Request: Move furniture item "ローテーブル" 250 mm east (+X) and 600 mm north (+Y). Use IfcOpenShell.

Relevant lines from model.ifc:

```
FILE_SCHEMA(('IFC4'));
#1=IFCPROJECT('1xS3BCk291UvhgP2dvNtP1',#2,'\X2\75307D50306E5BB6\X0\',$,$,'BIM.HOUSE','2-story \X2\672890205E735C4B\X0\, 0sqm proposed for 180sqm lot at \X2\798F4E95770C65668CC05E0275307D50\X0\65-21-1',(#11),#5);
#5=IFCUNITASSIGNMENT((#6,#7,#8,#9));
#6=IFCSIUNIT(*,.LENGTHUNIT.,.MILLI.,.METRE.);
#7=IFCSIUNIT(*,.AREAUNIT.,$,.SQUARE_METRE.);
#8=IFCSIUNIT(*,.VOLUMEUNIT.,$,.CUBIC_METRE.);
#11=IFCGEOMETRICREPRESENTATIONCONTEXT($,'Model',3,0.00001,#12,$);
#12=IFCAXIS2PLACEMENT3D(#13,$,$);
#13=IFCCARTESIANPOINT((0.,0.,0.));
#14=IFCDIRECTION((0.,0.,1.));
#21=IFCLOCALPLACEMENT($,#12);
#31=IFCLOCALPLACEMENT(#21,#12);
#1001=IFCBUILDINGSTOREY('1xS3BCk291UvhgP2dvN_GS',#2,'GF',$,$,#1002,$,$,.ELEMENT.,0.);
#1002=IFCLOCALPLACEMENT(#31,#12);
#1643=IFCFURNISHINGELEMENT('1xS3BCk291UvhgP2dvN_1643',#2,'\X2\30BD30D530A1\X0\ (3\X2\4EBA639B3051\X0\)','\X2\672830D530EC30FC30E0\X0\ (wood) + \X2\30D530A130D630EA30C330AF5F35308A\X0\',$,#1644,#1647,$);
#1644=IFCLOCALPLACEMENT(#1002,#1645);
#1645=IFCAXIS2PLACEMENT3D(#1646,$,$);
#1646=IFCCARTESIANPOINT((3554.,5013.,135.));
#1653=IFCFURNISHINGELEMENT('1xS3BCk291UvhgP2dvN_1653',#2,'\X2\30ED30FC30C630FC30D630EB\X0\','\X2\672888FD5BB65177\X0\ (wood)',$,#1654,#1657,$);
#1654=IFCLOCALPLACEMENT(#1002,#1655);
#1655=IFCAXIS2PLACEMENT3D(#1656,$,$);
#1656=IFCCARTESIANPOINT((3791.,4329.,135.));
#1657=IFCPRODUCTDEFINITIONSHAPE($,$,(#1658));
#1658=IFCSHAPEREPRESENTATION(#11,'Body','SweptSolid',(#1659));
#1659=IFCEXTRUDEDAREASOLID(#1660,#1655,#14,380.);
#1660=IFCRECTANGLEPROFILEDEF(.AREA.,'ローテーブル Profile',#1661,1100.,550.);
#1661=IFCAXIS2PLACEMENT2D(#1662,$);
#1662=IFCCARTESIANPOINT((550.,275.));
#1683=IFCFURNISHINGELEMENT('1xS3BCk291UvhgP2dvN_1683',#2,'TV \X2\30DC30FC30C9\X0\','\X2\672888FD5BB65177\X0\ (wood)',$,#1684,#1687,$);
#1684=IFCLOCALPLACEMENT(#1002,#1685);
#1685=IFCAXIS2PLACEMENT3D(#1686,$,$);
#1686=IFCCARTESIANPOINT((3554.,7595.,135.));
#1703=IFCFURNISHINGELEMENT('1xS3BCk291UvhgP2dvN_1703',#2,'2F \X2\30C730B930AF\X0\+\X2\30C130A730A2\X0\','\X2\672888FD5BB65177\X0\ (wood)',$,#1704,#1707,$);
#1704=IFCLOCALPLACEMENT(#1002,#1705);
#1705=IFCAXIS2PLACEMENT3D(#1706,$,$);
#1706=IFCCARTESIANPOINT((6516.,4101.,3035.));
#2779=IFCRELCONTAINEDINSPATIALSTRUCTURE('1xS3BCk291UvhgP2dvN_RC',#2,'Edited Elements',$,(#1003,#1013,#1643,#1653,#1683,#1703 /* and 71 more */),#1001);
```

```python
import ifcopenshell
import ifcopenshell.api.geometry
import ifcopenshell.util.placement
import ifcopenshell.util.unit

model = ifcopenshell.open("model.ifc")
unit_scale = ifcopenshell.util.unit.calculate_unit_scale(model)

item = model.by_id(1653)
matrix = ifcopenshell.util.placement.get_local_placement(item.ObjectPlacement)
matrix[0, 3] += 0.25 / unit_scale
matrix[1, 3] += 0.6 / unit_scale
ifcopenshell.api.geometry.edit_object_placement(model, product=item, matrix=matrix, is_si=False)

print(ifcopenshell.util.placement.get_local_placement(item.ObjectPlacement).round(3) + 0.0)

model.write("model_rev.ifc")
```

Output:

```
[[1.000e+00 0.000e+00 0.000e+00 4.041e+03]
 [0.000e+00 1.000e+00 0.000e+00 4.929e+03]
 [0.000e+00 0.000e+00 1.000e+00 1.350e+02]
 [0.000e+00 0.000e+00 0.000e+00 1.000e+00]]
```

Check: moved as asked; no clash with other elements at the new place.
